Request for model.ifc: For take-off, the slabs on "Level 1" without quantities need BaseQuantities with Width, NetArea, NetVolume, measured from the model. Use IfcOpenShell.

First a look at what the model holds.

```python
import ifcopenshell
import ifcopenshell.util.element
import ifcopenshell.util.unit

model = ifcopenshell.open("model.ifc")
print(model.schema)
for unit_type in ("LENGTHUNIT", "AREAUNIT", "VOLUMEUNIT"):
    print(unit_type, ifcopenshell.util.unit.calculate_unit_scale(model, unit_type))
storey = next(s for s in model.by_type("IfcBuildingStorey") if s.Name == "Level 1")
slabs = [e for e in ifcopenshell.util.element.get_decomposition(storey) if e.is_a("IfcSlab")]
for e in sorted(slabs, key=lambda e: e.id()):
    print(e.id(), e.is_a(), e.Name, list(ifcopenshell.util.element.get_psets(e, qtos_only=True)), sep=" | ")
```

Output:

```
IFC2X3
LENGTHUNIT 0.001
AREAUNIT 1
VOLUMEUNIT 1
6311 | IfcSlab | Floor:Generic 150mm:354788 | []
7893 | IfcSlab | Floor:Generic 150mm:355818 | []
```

```python
import ifcopenshell
import ifcopenshell.api.pset
import ifcopenshell.geom
import ifcopenshell.util.element
import ifcopenshell.util.shape
import ifcopenshell.util.unit

model = ifcopenshell.open("model.ifc")
unit_scale = ifcopenshell.util.unit.calculate_unit_scale(model)
area_scale = ifcopenshell.util.unit.calculate_unit_scale(model, "AREAUNIT")
volume_scale = ifcopenshell.util.unit.calculate_unit_scale(model, "VOLUMEUNIT")
settings = ifcopenshell.geom.settings()

storey = next(s for s in model.by_type("IfcBuildingStorey") if s.Name == "Level 1")
slabs = [e for e in ifcopenshell.util.element.get_decomposition(storey) if e.is_a("IfcSlab")]

for e in sorted(slabs, key=lambda e: e.id()):
    if ifcopenshell.util.element.get_psets(e, qtos_only=True, should_inherit=False):
        continue
    # Geometry comes back in metres, in the element's own axes.
    shape = ifcopenshell.geom.create_shape(settings, e)
    values = {
        "Width": ifcopenshell.util.shape.get_z(shape.geometry) / unit_scale,
        "NetArea": ifcopenshell.util.shape.get_footprint_area(shape.geometry) / area_scale,
        "NetVolume": ifcopenshell.util.shape.get_volume(shape.geometry) / volume_scale,
    }
    qto = ifcopenshell.api.pset.add_qto(model, product=e, name="BaseQuantities")
    ifcopenshell.api.pset.edit_qto(model, qto=qto, properties=values)
    print(e.id(), {k: round(v, 3) for k, v in values.items()})

model.write("model_v2.ifc")
```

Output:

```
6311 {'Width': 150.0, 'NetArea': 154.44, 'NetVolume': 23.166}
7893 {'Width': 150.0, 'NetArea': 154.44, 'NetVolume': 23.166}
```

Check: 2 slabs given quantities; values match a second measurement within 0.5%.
